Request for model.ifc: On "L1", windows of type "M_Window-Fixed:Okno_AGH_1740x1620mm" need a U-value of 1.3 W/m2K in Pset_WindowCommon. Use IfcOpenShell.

First a look at what the model holds.

```python
import ifcopenshell
import ifcopenshell.util.element

model = ifcopenshell.open("model.ifc")
print(model.schema)
storey = next(s for s in model.by_type("IfcBuildingStorey") if s.Name == "L1")
windows = [e for e in ifcopenshell.util.element.get_decomposition(storey) if e.is_a("IfcWindow")]
seen = {}
for e in windows:
    element_type = ifcopenshell.util.element.get_type(e)
    key = (element_type.Name if element_type != e and element_type else None, ifcopenshell.util.element.get_pset(e, "Pset_WindowCommon", "ThermalTransmittance"))
    seen[key] = seen.get(key, 0) + 1
for (name, value), count in sorted(seen.items(), key=str):
    print(count, "x", name, "|", value)
```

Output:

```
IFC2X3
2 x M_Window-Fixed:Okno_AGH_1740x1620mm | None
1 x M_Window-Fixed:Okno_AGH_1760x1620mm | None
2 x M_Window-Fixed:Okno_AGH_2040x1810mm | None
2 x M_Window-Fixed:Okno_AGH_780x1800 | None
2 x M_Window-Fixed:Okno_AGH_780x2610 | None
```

```python
import ifcopenshell
import ifcopenshell.api.pset
import ifcopenshell.util.element

model = ifcopenshell.open("model.ifc")

storey = next(s for s in model.by_type("IfcBuildingStorey") if s.Name == "L1")
windows = [e for e in ifcopenshell.util.element.get_decomposition(storey) if e.is_a("IfcWindow")]

count = 0
for e in windows:
    element_type = ifcopenshell.util.element.get_type(e)
    if element_type in (None, e) or element_type.Name != "M_Window-Fixed:Okno_AGH_1740x1620mm":
        continue
    # add_pset returns the element's existing set when there is one.
    pset = ifcopenshell.api.pset.add_pset(model, product=e, name="Pset_WindowCommon")
    ifcopenshell.api.pset.edit_pset(model, pset=pset, properties={"ThermalTransmittance": 1.3})
    count += 1

print(count, "windows updated")

model.write("model_v2.ifc")
```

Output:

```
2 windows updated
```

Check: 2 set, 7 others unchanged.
